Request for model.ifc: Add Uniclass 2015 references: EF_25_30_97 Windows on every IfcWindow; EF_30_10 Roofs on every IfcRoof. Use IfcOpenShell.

First a look at what the model holds.

```python
import ifcopenshell

model = ifcopenshell.open("model.ifc")
print(model.schema)
print("classifications:", [c.Name for c in model.by_type("IfcClassification")])
for ifc_class in ("IfcDoor", "IfcRoof", "IfcStair", "IfcWall", "IfcWindow"):
    print(ifc_class, len(model.by_type(ifc_class)))
```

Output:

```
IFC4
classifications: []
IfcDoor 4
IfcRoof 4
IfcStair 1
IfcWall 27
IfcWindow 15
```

```python
import ifcopenshell
import ifcopenshell.api.classification

model = ifcopenshell.open("model.ifc")

system = ifcopenshell.api.classification.add_classification(model, classification="Uniclass 2015")

codes = {
    "IfcWindow": ("EF_25_30_97", "Windows"),
    "IfcRoof": ("EF_30_10", "Roofs"),
}
for ifc_class, (code, name) in codes.items():
    products = model.by_type(ifc_class)
    ifcopenshell.api.classification.add_reference(
        model, products=products, classification=system, identification=code, name=name
    )
    print(code, len(products))

model.write("model-out.ifc")
```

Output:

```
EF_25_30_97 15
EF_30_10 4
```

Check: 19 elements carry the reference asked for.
